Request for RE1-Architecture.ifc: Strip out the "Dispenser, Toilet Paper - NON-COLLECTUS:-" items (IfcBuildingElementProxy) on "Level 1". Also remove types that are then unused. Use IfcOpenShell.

First a look at what the model holds.

```python
import ifcopenshell
import ifcopenshell.util.element

model = ifcopenshell.open("RE1-Architecture.ifc")
print(model.schema)
storey = next(s for s in model.by_type("IfcBuildingStorey") if s.Name == "Level 1")
proxies = [e for e in ifcopenshell.util.element.get_decomposition(storey) if e.is_a("IfcBuildingElementProxy")]
seen = {}
for e in proxies:
    element_type = ifcopenshell.util.element.get_type(e)
    name = element_type.Name if element_type not in (None, e) else None
    seen[name] = seen.get(name, 0) + 1
for name, count in sorted(seen.items(), key=str):
    print(count, "x", name)
```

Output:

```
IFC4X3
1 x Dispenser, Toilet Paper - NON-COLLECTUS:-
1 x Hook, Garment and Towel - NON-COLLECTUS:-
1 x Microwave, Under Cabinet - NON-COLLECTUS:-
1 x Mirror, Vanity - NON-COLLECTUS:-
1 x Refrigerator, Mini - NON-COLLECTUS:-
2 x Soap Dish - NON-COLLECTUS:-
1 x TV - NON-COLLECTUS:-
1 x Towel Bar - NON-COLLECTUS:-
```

```python
import ifcopenshell
import ifcopenshell.api.root
import ifcopenshell.util.element

model = ifcopenshell.open("RE1-Architecture.ifc")

storey = next(s for s in model.by_type("IfcBuildingStorey") if s.Name == "Level 1")
proxies = [e for e in ifcopenshell.util.element.get_decomposition(storey) if e.is_a("IfcBuildingElementProxy")]
targets = [e for e in proxies if (t := ifcopenshell.util.element.get_type(e)) not in (None, e) and t.Name == "Dispenser, Toilet Paper - NON-COLLECTUS:-"]
types = {ifcopenshell.util.element.get_type(e) for e in targets} - {None, *targets}

for e in targets:
    ifcopenshell.api.root.remove_product(model, product=e)
print(len(targets), "removed")

unused = [t for t in types if not ifcopenshell.util.element.get_types(t)]
for t in unused:
    ifcopenshell.api.root.remove_product(model, product=t)
print(len(unused), "unused types removed")

model.write("RE1-Architecture_edited.ifc")
```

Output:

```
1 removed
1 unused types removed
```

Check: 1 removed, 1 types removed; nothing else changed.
